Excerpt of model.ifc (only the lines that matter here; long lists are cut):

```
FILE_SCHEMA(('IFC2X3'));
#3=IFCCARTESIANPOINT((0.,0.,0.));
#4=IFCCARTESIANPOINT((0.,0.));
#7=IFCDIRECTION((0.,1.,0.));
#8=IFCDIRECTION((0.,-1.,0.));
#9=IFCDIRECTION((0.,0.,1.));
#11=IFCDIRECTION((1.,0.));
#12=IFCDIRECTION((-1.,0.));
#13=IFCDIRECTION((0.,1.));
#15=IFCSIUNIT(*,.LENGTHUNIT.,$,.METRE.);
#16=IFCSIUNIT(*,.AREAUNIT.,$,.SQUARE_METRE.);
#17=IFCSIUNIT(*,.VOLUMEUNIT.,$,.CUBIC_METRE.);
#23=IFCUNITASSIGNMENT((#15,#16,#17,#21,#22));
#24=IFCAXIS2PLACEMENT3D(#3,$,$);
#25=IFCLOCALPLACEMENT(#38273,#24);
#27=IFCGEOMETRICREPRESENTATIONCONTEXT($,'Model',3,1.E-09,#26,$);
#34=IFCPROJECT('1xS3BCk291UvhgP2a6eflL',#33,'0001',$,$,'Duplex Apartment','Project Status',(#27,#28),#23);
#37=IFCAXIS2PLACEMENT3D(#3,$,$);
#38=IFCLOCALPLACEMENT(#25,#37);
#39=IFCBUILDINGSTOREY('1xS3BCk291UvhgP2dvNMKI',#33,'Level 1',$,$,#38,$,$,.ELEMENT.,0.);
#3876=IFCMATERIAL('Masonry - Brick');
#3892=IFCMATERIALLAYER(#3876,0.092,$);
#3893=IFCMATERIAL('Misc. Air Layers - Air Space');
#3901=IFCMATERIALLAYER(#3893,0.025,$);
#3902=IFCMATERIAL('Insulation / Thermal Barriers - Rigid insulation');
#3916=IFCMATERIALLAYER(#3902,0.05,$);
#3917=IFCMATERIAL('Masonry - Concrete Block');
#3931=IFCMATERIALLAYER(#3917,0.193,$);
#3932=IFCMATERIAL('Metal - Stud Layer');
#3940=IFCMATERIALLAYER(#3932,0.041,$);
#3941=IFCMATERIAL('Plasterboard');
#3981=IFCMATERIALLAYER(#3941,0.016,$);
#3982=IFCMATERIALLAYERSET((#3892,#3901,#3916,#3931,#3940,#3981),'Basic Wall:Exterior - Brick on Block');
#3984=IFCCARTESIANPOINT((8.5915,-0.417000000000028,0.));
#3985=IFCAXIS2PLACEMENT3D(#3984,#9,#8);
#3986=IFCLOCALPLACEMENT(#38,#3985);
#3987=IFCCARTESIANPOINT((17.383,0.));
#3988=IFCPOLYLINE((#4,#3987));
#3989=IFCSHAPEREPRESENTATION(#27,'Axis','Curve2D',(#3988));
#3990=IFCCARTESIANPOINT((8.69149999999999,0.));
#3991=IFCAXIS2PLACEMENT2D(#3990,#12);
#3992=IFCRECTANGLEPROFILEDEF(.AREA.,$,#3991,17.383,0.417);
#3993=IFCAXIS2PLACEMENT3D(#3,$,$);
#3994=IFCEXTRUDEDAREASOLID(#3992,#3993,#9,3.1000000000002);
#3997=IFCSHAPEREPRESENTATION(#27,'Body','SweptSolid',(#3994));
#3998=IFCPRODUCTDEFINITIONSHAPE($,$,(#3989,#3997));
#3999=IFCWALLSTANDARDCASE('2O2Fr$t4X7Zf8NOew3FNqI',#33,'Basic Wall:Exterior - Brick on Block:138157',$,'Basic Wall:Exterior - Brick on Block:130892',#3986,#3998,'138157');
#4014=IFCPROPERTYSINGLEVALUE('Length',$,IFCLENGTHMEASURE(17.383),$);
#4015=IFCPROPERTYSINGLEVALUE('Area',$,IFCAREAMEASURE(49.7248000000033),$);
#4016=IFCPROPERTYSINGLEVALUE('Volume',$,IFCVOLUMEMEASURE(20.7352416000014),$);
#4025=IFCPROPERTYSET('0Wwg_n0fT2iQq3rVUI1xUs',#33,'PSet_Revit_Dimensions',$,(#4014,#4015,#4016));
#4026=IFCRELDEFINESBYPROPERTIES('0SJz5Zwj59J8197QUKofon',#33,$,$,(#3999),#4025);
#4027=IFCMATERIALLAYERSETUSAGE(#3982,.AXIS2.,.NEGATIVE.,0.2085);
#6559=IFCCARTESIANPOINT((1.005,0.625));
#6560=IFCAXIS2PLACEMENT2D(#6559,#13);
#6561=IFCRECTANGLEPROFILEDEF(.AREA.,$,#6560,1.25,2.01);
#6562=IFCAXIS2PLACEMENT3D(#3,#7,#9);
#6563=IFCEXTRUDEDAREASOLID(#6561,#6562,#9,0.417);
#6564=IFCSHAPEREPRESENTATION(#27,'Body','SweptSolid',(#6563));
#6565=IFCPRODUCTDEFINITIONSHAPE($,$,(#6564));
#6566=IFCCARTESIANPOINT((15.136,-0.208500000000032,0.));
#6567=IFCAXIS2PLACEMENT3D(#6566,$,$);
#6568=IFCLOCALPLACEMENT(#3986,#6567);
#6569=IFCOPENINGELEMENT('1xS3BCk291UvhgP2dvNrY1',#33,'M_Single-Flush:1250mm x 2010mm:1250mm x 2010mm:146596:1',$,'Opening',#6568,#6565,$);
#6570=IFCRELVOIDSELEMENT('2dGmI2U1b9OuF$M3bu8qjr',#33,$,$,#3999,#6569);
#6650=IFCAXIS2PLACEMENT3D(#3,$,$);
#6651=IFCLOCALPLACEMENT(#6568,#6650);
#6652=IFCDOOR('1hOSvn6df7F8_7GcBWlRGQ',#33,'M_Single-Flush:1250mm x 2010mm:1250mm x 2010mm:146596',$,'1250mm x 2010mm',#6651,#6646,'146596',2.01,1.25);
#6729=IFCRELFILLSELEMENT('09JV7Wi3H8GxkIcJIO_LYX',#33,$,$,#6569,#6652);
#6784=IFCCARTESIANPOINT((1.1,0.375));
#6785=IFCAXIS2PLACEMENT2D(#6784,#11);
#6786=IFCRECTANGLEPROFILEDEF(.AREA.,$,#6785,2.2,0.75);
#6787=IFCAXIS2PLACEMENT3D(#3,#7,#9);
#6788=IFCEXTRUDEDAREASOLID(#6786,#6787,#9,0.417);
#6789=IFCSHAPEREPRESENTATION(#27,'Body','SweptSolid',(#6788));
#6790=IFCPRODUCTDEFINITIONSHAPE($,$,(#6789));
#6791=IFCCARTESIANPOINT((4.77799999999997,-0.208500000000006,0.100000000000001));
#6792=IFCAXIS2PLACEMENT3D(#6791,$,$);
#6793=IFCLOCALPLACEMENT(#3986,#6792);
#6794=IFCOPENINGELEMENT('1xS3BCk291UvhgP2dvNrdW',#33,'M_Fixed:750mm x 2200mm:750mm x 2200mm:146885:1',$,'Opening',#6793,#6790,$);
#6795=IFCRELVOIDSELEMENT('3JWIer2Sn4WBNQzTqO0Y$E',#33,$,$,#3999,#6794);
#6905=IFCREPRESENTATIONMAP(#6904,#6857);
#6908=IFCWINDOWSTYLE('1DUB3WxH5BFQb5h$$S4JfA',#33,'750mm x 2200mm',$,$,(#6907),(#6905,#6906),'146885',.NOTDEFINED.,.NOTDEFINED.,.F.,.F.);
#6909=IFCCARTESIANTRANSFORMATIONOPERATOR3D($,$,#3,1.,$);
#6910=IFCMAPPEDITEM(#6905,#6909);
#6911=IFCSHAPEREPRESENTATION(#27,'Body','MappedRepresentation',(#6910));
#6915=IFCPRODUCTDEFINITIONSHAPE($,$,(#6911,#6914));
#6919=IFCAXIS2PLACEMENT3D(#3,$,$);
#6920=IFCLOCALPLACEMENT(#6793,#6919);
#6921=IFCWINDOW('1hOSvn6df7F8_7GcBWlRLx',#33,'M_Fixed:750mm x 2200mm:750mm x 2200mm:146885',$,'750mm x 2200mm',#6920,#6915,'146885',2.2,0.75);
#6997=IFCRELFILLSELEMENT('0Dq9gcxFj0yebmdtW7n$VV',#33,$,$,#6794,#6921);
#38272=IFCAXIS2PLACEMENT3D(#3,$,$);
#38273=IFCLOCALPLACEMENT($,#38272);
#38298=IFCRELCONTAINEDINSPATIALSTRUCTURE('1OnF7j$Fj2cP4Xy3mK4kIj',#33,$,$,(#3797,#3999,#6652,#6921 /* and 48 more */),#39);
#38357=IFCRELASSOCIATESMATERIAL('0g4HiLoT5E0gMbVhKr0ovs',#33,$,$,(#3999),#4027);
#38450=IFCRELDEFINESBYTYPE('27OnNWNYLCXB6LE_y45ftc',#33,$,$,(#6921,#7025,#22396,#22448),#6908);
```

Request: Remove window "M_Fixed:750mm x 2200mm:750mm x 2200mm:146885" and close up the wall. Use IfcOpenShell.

```python
import ifcopenshell
import ifcopenshell.api.feature
import ifcopenshell.api.pset
import ifcopenshell.api.root
import ifcopenshell.geom
import ifcopenshell.util.element
import ifcopenshell.util.shape
import ifcopenshell.util.unit

model = ifcopenshell.open("model.ifc")
area_scale = ifcopenshell.util.unit.calculate_unit_scale(model, "AREAUNIT")
volume_scale = ifcopenshell.util.unit.calculate_unit_scale(model, "VOLUMEUNIT")
settings = ifcopenshell.geom.settings()


def volume(element):
    """Net volume in cubic metres, openings subtracted."""
    shape = ifcopenshell.geom.create_shape(settings, element)
    return ifcopenshell.util.shape.get_volume(shape.geometry)


window = model.by_id(6921)
opening = window.FillsVoids[0].RelatingOpeningElement
wall = opening.VoidsElements[0].RelatingBuildingElement
before = volume(wall)

ifcopenshell.api.root.remove_product(model, product=window)
ifcopenshell.api.feature.remove_feature(model, feature=opening)

after = volume(wall)
thickness = 0.417  # wall thickness in metres

# Update the wall's stored quantities.
pset = model.by_id(ifcopenshell.util.element.get_pset(wall, "PSet_Revit_Dimensions", should_inherit=False)["id"])
ifcopenshell.api.pset.edit_pset(model, pset=pset, properties={
    "Area": model.create_entity("IfcAreaMeasure", after / thickness / area_scale),
    "Volume": model.create_entity("IfcVolumeMeasure", after / volume_scale),
})

print(f"wall volume {before:.3f} -> {after:.3f} m3")

model.write("model-out.ifc")
```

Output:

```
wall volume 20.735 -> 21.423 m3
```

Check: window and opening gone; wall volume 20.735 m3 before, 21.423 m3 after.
